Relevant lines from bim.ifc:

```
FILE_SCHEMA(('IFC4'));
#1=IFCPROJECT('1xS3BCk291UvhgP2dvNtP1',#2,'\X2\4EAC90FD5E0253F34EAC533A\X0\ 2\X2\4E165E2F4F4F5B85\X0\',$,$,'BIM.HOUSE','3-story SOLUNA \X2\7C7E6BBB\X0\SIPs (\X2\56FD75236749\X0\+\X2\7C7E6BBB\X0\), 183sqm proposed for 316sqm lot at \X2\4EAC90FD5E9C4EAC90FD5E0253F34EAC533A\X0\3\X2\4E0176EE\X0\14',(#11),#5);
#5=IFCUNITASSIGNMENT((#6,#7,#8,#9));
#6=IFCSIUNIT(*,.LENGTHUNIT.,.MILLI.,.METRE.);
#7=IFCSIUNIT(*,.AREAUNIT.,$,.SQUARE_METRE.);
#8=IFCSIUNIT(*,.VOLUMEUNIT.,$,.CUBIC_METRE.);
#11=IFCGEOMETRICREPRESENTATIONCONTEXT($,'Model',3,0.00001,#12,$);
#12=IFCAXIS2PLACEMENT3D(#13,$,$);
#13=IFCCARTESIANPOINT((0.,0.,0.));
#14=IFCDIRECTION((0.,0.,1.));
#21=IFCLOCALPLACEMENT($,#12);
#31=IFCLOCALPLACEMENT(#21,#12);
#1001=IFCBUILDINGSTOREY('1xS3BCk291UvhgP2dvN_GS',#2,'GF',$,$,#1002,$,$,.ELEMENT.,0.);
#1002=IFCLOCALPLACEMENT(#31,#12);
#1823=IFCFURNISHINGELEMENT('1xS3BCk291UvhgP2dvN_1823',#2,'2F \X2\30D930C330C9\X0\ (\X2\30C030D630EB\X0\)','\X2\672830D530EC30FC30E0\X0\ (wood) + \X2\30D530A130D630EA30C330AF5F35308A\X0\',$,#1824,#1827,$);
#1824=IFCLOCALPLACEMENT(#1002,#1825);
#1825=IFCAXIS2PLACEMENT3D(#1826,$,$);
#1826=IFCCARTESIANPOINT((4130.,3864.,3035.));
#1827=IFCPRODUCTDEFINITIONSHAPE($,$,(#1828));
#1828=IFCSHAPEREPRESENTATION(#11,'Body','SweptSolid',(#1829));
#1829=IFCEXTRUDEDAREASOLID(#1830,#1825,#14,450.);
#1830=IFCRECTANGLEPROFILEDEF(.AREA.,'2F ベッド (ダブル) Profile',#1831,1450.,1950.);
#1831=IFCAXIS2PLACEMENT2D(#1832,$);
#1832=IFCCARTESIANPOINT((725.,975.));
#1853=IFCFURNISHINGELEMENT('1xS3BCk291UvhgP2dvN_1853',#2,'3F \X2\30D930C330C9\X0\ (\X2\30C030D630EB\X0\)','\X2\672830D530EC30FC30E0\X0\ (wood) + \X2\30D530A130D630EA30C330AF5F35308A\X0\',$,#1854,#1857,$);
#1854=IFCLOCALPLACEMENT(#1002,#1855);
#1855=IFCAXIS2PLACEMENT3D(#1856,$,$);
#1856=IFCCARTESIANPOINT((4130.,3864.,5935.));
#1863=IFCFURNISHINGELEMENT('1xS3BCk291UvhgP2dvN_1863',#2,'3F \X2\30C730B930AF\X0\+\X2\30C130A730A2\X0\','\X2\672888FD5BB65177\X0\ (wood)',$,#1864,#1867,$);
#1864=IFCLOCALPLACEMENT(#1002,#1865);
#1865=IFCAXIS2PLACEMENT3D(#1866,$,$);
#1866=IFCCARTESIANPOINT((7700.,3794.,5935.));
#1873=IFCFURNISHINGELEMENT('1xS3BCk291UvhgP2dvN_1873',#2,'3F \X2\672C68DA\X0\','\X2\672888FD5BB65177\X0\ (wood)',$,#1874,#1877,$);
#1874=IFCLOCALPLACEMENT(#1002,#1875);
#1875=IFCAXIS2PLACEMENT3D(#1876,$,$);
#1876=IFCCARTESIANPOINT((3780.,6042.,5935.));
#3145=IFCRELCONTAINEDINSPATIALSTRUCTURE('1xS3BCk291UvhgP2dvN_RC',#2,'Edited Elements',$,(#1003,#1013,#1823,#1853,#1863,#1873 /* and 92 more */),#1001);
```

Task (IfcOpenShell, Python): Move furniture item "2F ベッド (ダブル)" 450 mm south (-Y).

```python
import ifcopenshell
import ifcopenshell.api.geometry
import ifcopenshell.util.placement
import ifcopenshell.util.unit

model = ifcopenshell.open("bim.ifc")
unit_scale = ifcopenshell.util.unit.calculate_unit_scale(model)

item = model.by_id(1823)
matrix = ifcopenshell.util.placement.get_local_placement(item.ObjectPlacement)
matrix[1, 3] -= 0.45 / unit_scale
ifcopenshell.api.geometry.edit_object_placement(model, product=item, matrix=matrix, is_si=False)

print(ifcopenshell.util.placement.get_local_placement(item.ObjectPlacement).round(3) + 0.0)

model.write("bim_rev.ifc")
```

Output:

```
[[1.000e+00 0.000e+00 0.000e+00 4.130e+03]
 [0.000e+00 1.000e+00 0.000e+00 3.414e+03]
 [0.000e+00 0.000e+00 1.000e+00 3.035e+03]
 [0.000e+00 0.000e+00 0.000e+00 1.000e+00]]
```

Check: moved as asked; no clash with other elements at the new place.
